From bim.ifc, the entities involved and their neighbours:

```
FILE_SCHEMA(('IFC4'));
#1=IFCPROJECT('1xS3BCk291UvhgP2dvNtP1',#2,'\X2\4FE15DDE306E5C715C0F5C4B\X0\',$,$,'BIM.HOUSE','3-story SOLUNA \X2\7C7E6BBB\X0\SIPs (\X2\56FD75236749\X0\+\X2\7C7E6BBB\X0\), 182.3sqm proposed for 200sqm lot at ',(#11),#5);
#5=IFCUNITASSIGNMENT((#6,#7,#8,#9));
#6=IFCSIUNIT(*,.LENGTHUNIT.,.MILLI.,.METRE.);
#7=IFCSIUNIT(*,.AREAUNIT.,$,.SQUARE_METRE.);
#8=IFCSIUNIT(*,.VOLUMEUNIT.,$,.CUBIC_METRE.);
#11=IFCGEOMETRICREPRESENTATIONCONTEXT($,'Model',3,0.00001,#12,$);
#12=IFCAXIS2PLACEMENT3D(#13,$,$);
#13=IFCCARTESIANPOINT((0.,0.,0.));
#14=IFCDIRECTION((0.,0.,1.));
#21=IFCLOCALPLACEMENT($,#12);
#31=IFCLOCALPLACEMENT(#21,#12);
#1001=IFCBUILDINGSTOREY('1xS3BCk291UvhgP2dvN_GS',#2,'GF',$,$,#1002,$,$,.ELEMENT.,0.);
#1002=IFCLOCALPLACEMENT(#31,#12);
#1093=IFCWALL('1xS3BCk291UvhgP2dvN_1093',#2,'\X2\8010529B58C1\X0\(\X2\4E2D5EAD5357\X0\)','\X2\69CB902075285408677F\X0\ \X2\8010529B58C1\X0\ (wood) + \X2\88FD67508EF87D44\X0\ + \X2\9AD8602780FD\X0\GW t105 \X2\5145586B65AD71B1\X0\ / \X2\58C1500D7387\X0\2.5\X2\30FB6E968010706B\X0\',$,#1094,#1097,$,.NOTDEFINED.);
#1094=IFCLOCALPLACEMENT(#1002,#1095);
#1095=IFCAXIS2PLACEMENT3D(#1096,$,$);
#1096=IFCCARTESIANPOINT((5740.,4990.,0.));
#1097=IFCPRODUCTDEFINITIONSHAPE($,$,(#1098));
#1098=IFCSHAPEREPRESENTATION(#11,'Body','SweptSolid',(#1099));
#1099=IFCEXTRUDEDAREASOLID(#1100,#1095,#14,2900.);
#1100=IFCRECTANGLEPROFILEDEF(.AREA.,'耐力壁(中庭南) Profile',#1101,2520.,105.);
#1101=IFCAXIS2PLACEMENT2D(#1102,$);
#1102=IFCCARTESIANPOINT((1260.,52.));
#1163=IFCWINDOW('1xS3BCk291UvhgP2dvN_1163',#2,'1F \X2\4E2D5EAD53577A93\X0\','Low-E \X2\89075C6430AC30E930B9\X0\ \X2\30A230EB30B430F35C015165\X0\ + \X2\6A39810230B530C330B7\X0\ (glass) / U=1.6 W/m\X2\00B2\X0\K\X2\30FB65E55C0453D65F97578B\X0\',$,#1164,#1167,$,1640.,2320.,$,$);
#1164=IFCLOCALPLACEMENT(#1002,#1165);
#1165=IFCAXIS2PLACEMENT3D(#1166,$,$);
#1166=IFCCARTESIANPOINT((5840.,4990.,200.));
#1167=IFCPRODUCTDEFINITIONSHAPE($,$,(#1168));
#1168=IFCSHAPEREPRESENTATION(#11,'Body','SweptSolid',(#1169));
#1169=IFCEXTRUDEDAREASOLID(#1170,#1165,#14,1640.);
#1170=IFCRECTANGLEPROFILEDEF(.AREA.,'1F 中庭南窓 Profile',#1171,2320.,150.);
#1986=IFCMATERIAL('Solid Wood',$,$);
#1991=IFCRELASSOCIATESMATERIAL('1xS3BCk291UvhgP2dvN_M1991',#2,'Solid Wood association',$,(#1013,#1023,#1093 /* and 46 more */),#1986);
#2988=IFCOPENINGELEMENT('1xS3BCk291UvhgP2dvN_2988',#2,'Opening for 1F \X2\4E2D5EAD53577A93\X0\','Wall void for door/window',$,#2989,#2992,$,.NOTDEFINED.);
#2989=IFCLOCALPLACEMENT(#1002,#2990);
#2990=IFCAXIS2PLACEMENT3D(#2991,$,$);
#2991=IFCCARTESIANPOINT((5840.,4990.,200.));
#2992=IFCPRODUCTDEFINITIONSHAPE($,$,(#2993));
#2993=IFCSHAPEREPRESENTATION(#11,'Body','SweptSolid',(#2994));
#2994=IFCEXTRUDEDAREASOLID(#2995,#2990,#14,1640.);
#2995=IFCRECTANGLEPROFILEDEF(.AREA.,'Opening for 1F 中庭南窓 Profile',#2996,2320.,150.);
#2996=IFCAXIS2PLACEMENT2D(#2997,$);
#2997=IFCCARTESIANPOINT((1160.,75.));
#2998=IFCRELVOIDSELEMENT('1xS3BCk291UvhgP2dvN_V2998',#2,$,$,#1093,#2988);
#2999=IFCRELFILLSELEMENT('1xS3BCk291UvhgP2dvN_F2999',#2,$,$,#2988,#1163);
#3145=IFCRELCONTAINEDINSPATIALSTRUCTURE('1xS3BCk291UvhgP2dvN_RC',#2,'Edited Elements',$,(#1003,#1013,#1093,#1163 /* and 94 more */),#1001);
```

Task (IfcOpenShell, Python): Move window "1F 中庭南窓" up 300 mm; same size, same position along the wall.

```python
import numpy as np
import ifcopenshell
import ifcopenshell.api.geometry
import ifcopenshell.util.placement
import ifcopenshell.util.unit

model = ifcopenshell.open("bim.ifc")
unit_scale = ifcopenshell.util.unit.calculate_unit_scale(model)

window = model.by_guid("1xS3BCk291UvhgP2dvN_1163")
opening = window.FillsVoids[0].RelatingOpeningElement
dz = 0.3 / unit_scale

shift = np.array([0.0, 0.0, dz])
# The window is not placed relative to its opening, so move both.
for product in (opening, window):
    matrix = ifcopenshell.util.placement.get_local_placement(product.ObjectPlacement)
    matrix[:3, 3] += shift
    ifcopenshell.api.geometry.edit_object_placement(model, product=product, matrix=matrix, is_si=False)

print(f"moved by {dz * unit_scale:+.3f} m")

model.write("bim_updated.ifc")
```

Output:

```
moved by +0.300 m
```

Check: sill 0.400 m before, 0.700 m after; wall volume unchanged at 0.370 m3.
